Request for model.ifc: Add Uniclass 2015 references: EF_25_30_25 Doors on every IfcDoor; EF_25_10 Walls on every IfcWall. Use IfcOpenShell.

First a look at what the model holds.

```python
import ifcopenshell

model = ifcopenshell.open("model.ifc")
print(model.schema)
print("classifications:", [c.Name for c in model.by_type("IfcClassification")])
for ifc_class in ("IfcDoor", "IfcRoof", "IfcStair", "IfcWall", "IfcWindow"):
    print(ifc_class, len(model.by_type(ifc_class)))
```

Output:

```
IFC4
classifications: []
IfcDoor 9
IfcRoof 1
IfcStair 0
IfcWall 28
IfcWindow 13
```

```python
import ifcopenshell
import ifcopenshell.api.classification

model = ifcopenshell.open("model.ifc")

system = ifcopenshell.api.classification.add_classification(model, classification="Uniclass 2015")

codes = {
    "IfcDoor": ("EF_25_30_25", "Doors"),
    "IfcWall": ("EF_25_10", "Walls"),
}
for ifc_class, (code, name) in codes.items():
    products = model.by_type(ifc_class)
    ifcopenshell.api.classification.add_reference(
        model, products=products, classification=system, identification=code, name=name
    )
    print(code, len(products))

model.write("model_rev.ifc")
```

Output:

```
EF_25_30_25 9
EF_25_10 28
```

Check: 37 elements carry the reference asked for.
